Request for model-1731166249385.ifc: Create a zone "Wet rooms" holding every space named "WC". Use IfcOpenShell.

First a look at what the model holds.

```python
import ifcopenshell

model = ifcopenshell.open("model-1731166249385.ifc")
print(model.schema)
seen = {}
for space in model.by_type("IfcSpace"):
    seen[space.LongName] = seen.get(space.LongName, 0) + 1
for name, count in sorted(seen.items(), key=str):
    print(count, "x", name)
print("zones:", [z.Name for z in model.by_type("IfcZone")][:20])
```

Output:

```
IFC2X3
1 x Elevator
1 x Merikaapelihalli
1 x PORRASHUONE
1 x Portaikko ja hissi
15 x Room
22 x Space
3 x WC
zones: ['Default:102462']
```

```python
import ifcopenshell
import ifcopenshell.api.group
import ifcopenshell.api.root

model = ifcopenshell.open("model-1731166249385.ifc")

names = {"WC"}
spaces = [s for s in model.by_type("IfcSpace") if s.LongName in names]

zone = ifcopenshell.api.root.create_entity(model, ifc_class="IfcZone", name="Wet rooms")
ifcopenshell.api.group.assign_group(model, products=spaces, group=zone)
print(len(spaces), "spaces in", zone.Name)

model.write("model-1731166249385_v2.ifc")
```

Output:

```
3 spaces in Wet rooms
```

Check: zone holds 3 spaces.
